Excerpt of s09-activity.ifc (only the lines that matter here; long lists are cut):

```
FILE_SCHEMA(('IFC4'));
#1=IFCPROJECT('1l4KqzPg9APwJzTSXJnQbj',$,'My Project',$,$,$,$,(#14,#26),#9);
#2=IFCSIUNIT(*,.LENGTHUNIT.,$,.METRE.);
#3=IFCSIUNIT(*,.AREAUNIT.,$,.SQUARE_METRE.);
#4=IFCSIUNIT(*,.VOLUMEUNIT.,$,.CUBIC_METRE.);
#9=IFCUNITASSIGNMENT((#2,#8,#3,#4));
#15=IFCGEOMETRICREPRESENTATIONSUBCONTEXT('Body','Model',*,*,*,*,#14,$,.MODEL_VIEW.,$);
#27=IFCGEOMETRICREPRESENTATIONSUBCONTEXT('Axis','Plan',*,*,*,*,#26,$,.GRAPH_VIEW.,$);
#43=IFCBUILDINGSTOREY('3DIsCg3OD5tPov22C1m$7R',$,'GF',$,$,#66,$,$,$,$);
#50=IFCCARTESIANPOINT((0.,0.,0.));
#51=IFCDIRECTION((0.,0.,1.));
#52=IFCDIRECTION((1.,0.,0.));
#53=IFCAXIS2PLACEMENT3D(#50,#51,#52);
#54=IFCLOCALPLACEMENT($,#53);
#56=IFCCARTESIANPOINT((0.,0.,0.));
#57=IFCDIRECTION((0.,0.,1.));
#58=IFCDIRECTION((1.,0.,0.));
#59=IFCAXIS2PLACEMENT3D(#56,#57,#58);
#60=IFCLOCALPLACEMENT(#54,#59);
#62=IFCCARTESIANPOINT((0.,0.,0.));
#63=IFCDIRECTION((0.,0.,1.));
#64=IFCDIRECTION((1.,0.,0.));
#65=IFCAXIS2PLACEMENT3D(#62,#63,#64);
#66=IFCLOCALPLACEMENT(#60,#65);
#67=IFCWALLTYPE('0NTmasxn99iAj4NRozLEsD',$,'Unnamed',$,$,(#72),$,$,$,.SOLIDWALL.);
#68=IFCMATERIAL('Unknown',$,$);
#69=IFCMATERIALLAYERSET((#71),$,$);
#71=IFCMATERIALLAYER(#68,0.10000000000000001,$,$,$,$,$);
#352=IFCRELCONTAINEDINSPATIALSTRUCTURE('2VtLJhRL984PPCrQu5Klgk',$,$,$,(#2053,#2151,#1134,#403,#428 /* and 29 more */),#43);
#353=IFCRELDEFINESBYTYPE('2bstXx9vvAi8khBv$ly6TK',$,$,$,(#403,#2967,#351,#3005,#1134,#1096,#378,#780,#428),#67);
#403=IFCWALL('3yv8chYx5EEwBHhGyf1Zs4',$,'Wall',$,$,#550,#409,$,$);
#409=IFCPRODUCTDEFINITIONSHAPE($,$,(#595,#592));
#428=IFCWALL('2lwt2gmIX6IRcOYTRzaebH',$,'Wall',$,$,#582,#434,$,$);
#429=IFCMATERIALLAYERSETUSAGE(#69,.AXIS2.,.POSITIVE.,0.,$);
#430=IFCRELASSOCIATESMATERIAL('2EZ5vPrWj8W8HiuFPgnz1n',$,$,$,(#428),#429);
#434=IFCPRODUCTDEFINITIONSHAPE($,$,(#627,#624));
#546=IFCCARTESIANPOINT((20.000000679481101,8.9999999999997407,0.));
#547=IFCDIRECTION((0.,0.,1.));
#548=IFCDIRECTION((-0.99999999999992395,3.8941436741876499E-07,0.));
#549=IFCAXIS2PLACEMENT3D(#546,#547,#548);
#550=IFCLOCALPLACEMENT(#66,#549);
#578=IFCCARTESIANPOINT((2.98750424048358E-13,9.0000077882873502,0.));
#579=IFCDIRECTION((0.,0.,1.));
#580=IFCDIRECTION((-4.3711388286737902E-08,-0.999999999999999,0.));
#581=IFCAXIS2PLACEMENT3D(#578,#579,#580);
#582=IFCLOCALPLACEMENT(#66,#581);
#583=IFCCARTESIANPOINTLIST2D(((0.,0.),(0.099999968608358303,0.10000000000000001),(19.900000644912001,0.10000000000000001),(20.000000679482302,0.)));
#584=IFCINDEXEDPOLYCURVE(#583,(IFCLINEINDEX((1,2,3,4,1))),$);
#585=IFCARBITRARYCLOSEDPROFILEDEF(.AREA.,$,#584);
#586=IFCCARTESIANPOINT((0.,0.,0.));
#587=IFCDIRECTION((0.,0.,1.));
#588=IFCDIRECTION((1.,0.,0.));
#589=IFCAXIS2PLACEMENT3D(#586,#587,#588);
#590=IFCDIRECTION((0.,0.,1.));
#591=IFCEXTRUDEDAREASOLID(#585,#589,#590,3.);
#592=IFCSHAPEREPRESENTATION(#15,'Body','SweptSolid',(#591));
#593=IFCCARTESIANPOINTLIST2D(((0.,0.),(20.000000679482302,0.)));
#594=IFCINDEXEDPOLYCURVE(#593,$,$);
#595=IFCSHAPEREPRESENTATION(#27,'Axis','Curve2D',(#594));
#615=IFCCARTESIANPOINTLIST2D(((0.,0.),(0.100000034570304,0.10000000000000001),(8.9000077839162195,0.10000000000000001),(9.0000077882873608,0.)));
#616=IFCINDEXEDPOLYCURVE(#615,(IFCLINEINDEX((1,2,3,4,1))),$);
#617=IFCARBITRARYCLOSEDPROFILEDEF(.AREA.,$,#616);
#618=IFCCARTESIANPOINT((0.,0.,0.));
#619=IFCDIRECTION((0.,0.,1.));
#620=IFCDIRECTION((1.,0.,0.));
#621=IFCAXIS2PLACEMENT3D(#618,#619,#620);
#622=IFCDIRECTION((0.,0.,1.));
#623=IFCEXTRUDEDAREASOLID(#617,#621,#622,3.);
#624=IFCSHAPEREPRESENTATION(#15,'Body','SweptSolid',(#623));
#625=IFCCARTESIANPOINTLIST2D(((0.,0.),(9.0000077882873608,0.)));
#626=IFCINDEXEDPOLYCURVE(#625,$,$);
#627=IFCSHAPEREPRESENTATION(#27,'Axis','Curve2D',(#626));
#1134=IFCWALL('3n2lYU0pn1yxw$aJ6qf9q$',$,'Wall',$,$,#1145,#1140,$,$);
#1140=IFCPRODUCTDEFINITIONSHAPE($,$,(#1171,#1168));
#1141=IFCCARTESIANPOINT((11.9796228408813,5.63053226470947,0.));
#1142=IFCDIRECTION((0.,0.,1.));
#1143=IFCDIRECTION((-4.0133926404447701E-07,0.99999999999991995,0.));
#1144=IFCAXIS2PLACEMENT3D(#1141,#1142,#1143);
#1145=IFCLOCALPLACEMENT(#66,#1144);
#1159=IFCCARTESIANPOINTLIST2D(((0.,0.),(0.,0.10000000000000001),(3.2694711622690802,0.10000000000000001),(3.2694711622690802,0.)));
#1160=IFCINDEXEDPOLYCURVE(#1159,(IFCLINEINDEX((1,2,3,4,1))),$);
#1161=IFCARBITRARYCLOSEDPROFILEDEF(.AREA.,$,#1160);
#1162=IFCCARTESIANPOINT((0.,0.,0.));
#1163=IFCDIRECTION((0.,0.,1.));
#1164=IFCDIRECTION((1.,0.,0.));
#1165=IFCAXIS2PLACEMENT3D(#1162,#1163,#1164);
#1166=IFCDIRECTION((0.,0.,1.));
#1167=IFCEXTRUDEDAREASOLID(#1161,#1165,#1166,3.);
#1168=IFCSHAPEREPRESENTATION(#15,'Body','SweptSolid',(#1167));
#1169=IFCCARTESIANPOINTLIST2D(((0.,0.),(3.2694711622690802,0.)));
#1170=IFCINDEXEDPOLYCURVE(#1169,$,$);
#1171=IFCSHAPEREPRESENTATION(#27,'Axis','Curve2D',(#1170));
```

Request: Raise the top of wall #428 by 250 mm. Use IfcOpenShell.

```python
import ifcopenshell
import ifcopenshell.geom
import ifcopenshell.util.representation
import ifcopenshell.util.shape
import ifcopenshell.util.unit

model = ifcopenshell.open("s09-activity.ifc")
unit_scale = ifcopenshell.util.unit.calculate_unit_scale(model)
settings = ifcopenshell.geom.settings()


def volume(element):
    """Net volume in cubic metres, openings subtracted."""
    shape = ifcopenshell.geom.create_shape(settings, element)
    return ifcopenshell.util.shape.get_volume(shape.geometry)


wall = model.by_guid("2lwt2gmIX6IRcOYTRzaebH")
before = volume(wall)

body = ifcopenshell.util.representation.get_representation(wall, "Model", "Body")
solid = body.Items[0]
old_height = solid.Depth
solid.Depth += 0.25 / unit_scale
after = volume(wall)

print(f"height {old_height:g} -> {solid.Depth:g}, volume {before:.3f} -> {after:.3f} m3")

model.write("s09-activity_edited.ifc")
```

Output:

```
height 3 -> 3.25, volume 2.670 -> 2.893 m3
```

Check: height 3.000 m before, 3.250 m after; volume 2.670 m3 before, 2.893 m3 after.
